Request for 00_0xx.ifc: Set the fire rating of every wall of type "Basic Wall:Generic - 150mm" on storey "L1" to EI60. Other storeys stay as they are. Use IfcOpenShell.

First a look at what the model holds.

```python
import ifcopenshell
import ifcopenshell.util.element

model = ifcopenshell.open("00_0xx.ifc")
print(model.schema)
storey = next(s for s in model.by_type("IfcBuildingStorey") if s.Name == "L1")
walls = [e for e in ifcopenshell.util.element.get_decomposition(storey) if e.is_a("IfcWall")]
seen = {}
for e in walls:
    element_type = ifcopenshell.util.element.get_type(e)
    key = (element_type.Name if element_type != e and element_type else None, ifcopenshell.util.element.get_pset(e, "Pset_WallCommon", "FireRating"))
    seen[key] = seen.get(key, 0) + 1
for (name, value), count in sorted(seen.items(), key=str):
    print(count, "x", name, "|", value)
```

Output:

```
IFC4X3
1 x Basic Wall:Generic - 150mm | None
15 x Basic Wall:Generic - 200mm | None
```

```python
import ifcopenshell
import ifcopenshell.api.pset
import ifcopenshell.util.element

model = ifcopenshell.open("00_0xx.ifc")

storey = next(s for s in model.by_type("IfcBuildingStorey") if s.Name == "L1")
walls = [e for e in ifcopenshell.util.element.get_decomposition(storey) if e.is_a("IfcWall")]

count = 0
for e in walls:
    element_type = ifcopenshell.util.element.get_type(e)
    if element_type in (None, e) or element_type.Name != "Basic Wall:Generic - 150mm":
        continue
    # add_pset returns the element's existing set when there is one.
    pset = ifcopenshell.api.pset.add_pset(model, product=e, name="Pset_WallCommon")
    ifcopenshell.api.pset.edit_pset(model, pset=pset, properties={"FireRating": "EI60"})
    count += 1

print(count, "walls updated")

model.write("00_0xx_rev.ifc")
```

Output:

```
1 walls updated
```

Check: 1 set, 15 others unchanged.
